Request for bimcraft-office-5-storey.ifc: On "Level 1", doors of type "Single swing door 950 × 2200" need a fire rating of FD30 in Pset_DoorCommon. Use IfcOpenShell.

First a look at what the model holds.

```python
import ifcopenshell
import ifcopenshell.util.element

model = ifcopenshell.open("bimcraft-office-5-storey.ifc")
print(model.schema)
storey = next(s for s in model.by_type("IfcBuildingStorey") if s.Name == "Level 1")
doors = [e for e in ifcopenshell.util.element.get_decomposition(storey) if e.is_a("IfcDoor")]
seen = {}
for e in doors:
    element_type = ifcopenshell.util.element.get_type(e)
    key = (element_type.Name if element_type != e and element_type else None, ifcopenshell.util.element.get_pset(e, "Pset_DoorCommon", "FireRating"))
    seen[key] = seen.get(key, 0) + 1
for (name, value), count in sorted(seen.items(), key=str):
    print(count, "x", name, "|", value)
```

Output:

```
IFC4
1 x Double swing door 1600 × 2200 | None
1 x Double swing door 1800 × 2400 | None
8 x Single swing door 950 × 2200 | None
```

```python
import ifcopenshell
import ifcopenshell.api.pset
import ifcopenshell.util.element

model = ifcopenshell.open("bimcraft-office-5-storey.ifc")

storey = next(s for s in model.by_type("IfcBuildingStorey") if s.Name == "Level 1")
doors = [e for e in ifcopenshell.util.element.get_decomposition(storey) if e.is_a("IfcDoor")]

count = 0
for e in doors:
    element_type = ifcopenshell.util.element.get_type(e)
    if element_type in (None, e) or element_type.Name != "Single swing door 950 × 2200":
        continue
    # add_pset returns the element's existing set when there is one.
    pset = ifcopenshell.api.pset.add_pset(model, product=e, name="Pset_DoorCommon")
    ifcopenshell.api.pset.edit_pset(model, pset=pset, properties={"FireRating": "FD30"})
    count += 1

print(count, "doors updated")

model.write("bimcraft-office-5-storey-out.ifc")
```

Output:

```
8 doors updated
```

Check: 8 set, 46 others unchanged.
